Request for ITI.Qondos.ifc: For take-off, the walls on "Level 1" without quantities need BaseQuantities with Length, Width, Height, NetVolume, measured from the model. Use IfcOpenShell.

First a look at what the model holds.

```python
import ifcopenshell
import ifcopenshell.util.element
import ifcopenshell.util.unit

model = ifcopenshell.open("ITI.Qondos.ifc")
print(model.schema)
for unit_type in ("LENGTHUNIT", "AREAUNIT", "VOLUMEUNIT"):
    print(unit_type, ifcopenshell.util.unit.calculate_unit_scale(model, unit_type))
storey = next(s for s in model.by_type("IfcBuildingStorey") if s.Name == "Level 1")
walls = [e for e in ifcopenshell.util.element.get_decomposition(storey) if e.is_a("IfcWall")]
for e in sorted(walls, key=lambda e: e.id()):
    print(e.id(), e.is_a(), e.Name, list(ifcopenshell.util.element.get_psets(e, qtos_only=True)), sep=" | ")
```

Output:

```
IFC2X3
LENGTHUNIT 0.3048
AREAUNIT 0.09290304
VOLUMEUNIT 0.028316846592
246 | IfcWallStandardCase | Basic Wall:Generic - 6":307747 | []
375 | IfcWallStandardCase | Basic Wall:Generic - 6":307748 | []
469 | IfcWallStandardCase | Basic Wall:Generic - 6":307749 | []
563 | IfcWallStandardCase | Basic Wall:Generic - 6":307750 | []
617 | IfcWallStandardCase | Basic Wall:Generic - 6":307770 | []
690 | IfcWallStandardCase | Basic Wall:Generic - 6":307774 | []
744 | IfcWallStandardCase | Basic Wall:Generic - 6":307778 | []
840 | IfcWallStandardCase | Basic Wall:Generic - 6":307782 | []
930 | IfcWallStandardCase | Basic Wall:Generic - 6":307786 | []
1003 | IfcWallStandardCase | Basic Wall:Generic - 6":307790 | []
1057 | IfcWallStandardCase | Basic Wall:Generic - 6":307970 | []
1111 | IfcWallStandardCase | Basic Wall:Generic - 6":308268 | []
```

```python
import ifcopenshell
import ifcopenshell.api.pset
import ifcopenshell.geom
import ifcopenshell.util.element
import ifcopenshell.util.shape
import ifcopenshell.util.unit

model = ifcopenshell.open("ITI.Qondos.ifc")
unit_scale = ifcopenshell.util.unit.calculate_unit_scale(model)
volume_scale = ifcopenshell.util.unit.calculate_unit_scale(model, "VOLUMEUNIT")
settings = ifcopenshell.geom.settings()

storey = next(s for s in model.by_type("IfcBuildingStorey") if s.Name == "Level 1")
walls = [e for e in ifcopenshell.util.element.get_decomposition(storey) if e.is_a("IfcWall")]

for e in sorted(walls, key=lambda e: e.id()):
    if ifcopenshell.util.element.get_psets(e, qtos_only=True, should_inherit=False):
        continue
    # Geometry comes back in metres, in the element's own axes.
    shape = ifcopenshell.geom.create_shape(settings, e)
    values = {
        "Length": ifcopenshell.util.shape.get_x(shape.geometry) / unit_scale,
        "Width": ifcopenshell.util.shape.get_y(shape.geometry) / unit_scale,
        "Height": ifcopenshell.util.shape.get_z(shape.geometry) / unit_scale,
        "NetVolume": ifcopenshell.util.shape.get_volume(shape.geometry) / volume_scale,
    }
    qto = ifcopenshell.api.pset.add_qto(model, product=e, name="BaseQuantities")
    ifcopenshell.api.pset.edit_qto(model, qto=qto, properties=values)
    print(e.id(), {k: round(v, 3) for k, v in values.items()})

model.write("ITI.Qondos_rev.ifc")
```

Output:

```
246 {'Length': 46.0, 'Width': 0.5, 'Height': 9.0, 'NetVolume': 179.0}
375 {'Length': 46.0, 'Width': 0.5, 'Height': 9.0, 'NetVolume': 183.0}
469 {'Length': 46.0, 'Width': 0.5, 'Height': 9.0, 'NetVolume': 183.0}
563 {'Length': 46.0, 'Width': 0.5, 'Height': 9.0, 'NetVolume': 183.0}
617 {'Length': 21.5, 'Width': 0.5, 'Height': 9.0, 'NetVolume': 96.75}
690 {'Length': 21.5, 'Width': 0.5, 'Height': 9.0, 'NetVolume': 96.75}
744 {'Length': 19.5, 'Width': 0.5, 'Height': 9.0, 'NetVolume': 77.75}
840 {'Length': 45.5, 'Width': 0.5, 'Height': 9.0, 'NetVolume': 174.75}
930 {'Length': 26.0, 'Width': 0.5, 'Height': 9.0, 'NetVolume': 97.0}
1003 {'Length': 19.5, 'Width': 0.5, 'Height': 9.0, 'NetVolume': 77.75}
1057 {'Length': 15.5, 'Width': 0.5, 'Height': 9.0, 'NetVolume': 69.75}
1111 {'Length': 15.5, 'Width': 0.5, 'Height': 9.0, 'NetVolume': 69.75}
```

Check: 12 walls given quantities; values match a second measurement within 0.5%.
